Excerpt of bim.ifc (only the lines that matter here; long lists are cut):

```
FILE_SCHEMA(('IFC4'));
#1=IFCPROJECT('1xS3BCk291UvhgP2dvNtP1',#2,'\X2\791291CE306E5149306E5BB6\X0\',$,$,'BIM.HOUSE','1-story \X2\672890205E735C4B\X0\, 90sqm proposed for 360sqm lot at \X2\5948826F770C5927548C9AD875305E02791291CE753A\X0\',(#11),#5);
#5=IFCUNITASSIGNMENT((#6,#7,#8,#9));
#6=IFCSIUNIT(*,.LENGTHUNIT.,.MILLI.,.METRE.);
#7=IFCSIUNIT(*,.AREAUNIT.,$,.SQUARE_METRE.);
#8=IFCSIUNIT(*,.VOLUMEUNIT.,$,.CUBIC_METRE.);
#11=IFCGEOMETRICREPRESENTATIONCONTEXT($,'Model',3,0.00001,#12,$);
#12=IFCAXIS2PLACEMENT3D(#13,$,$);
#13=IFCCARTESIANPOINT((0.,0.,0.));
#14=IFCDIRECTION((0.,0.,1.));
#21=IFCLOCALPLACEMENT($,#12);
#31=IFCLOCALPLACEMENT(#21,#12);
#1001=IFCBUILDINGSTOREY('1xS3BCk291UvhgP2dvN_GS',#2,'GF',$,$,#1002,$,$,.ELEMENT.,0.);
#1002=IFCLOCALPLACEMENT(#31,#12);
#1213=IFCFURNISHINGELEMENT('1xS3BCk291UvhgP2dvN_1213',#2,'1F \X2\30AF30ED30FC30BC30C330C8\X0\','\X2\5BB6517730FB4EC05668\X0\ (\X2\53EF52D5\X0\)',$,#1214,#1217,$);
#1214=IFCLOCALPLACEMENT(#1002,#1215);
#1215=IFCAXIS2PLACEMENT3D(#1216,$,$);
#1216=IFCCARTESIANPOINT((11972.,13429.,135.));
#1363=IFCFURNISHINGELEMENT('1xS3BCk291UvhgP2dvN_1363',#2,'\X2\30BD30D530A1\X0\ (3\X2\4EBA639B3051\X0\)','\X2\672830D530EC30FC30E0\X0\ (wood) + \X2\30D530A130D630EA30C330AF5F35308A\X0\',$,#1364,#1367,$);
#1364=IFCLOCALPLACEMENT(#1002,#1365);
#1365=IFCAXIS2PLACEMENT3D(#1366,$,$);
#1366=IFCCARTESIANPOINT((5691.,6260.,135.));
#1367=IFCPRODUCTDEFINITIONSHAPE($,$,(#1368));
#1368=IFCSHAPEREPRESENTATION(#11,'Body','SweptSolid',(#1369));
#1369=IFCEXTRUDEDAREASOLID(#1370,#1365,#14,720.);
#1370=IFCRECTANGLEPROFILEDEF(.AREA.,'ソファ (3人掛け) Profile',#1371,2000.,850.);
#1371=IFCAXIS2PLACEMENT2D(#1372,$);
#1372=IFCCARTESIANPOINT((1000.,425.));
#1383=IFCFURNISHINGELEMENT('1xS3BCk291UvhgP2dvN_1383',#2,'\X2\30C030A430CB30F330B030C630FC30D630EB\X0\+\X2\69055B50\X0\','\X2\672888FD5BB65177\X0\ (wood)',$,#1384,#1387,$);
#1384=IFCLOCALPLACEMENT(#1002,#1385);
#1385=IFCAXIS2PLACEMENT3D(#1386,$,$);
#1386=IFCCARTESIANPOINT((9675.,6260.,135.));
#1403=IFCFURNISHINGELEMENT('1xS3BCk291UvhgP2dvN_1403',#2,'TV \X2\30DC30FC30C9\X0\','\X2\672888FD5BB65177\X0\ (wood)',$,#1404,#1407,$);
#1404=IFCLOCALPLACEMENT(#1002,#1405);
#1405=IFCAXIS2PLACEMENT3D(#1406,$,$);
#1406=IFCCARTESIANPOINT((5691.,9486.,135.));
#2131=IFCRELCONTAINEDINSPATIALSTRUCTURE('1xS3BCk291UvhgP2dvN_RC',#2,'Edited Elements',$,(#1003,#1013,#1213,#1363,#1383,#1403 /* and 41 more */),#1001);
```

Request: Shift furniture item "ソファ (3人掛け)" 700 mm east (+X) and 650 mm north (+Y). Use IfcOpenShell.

```python
import ifcopenshell
import ifcopenshell.api.geometry
import ifcopenshell.util.placement
import ifcopenshell.util.unit

model = ifcopenshell.open("bim.ifc")
unit_scale = ifcopenshell.util.unit.calculate_unit_scale(model)

item = model.by_guid("1xS3BCk291UvhgP2dvN_1363")
matrix = ifcopenshell.util.placement.get_local_placement(item.ObjectPlacement)
matrix[0, 3] += 0.7 / unit_scale
matrix[1, 3] += 0.65 / unit_scale
ifcopenshell.api.geometry.edit_object_placement(model, product=item, matrix=matrix, is_si=False)

print(ifcopenshell.util.placement.get_local_placement(item.ObjectPlacement).round(3) + 0.0)

model.write("bim-out.ifc")
```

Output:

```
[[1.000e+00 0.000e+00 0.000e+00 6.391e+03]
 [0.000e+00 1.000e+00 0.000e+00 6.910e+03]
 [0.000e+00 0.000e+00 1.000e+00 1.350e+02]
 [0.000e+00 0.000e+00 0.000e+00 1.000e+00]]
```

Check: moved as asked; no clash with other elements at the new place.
